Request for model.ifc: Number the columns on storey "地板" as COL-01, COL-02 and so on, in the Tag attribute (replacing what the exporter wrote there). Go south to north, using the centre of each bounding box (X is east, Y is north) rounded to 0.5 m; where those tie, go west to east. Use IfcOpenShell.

First a look at what the model holds.

```python
import ifcopenshell
import ifcopenshell.util.element
import ifcopenshell.util.placement

model = ifcopenshell.open("model.ifc")
print(model.schema)
storey = next(s for s in model.by_type("IfcBuildingStorey") if s.Name == "地板")
columns = [e for e in ifcopenshell.util.element.get_decomposition(storey) if e.is_a("IfcColumn")]
for e in sorted(columns, key=lambda e: e.id()):
    origin = ifcopenshell.util.placement.get_local_placement(e.ObjectPlacement)[:3, 3]
    print(e.id(), e.Tag, e.Name, origin.round(2) + 0.0, sep=" | ")
```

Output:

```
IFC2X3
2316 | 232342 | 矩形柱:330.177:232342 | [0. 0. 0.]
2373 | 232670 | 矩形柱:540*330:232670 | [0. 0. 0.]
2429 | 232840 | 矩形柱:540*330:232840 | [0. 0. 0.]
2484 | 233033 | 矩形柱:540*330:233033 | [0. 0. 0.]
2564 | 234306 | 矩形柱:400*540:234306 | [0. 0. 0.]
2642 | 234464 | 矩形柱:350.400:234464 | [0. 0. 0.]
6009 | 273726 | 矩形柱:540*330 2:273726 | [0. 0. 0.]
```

```python
import ifcopenshell
import ifcopenshell.geom
import ifcopenshell.util.element
import ifcopenshell.util.shape

model = ifcopenshell.open("model.ifc")
settings = ifcopenshell.geom.settings()
settings.set("use-world-coords", True)


def centre(element):
    shape = ifcopenshell.geom.create_shape(settings, element)
    return ifcopenshell.util.shape.get_bbox_centroid(shape.geometry)


storey = next(s for s in model.by_type("IfcBuildingStorey") if s.Name == "地板")
columns = [e for e in ifcopenshell.util.element.get_decomposition(storey) if e.is_a("IfcColumn")]

# Insertion points can sit at a corner or the storey origin, so sort by the geometry (in metres).
centres = {e: centre(e) for e in columns}
columns.sort(key=lambda e: (round(centres[e][1] / 0.5), centres[e][0]))

for i, e in enumerate(columns, start=1):
    number = f"COL-{i:02d}"
    e.Tag = number
    print(e.id(), number)

model.write("model_v2.ifc")
```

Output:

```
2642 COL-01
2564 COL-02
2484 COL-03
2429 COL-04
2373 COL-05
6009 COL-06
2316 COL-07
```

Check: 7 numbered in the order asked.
